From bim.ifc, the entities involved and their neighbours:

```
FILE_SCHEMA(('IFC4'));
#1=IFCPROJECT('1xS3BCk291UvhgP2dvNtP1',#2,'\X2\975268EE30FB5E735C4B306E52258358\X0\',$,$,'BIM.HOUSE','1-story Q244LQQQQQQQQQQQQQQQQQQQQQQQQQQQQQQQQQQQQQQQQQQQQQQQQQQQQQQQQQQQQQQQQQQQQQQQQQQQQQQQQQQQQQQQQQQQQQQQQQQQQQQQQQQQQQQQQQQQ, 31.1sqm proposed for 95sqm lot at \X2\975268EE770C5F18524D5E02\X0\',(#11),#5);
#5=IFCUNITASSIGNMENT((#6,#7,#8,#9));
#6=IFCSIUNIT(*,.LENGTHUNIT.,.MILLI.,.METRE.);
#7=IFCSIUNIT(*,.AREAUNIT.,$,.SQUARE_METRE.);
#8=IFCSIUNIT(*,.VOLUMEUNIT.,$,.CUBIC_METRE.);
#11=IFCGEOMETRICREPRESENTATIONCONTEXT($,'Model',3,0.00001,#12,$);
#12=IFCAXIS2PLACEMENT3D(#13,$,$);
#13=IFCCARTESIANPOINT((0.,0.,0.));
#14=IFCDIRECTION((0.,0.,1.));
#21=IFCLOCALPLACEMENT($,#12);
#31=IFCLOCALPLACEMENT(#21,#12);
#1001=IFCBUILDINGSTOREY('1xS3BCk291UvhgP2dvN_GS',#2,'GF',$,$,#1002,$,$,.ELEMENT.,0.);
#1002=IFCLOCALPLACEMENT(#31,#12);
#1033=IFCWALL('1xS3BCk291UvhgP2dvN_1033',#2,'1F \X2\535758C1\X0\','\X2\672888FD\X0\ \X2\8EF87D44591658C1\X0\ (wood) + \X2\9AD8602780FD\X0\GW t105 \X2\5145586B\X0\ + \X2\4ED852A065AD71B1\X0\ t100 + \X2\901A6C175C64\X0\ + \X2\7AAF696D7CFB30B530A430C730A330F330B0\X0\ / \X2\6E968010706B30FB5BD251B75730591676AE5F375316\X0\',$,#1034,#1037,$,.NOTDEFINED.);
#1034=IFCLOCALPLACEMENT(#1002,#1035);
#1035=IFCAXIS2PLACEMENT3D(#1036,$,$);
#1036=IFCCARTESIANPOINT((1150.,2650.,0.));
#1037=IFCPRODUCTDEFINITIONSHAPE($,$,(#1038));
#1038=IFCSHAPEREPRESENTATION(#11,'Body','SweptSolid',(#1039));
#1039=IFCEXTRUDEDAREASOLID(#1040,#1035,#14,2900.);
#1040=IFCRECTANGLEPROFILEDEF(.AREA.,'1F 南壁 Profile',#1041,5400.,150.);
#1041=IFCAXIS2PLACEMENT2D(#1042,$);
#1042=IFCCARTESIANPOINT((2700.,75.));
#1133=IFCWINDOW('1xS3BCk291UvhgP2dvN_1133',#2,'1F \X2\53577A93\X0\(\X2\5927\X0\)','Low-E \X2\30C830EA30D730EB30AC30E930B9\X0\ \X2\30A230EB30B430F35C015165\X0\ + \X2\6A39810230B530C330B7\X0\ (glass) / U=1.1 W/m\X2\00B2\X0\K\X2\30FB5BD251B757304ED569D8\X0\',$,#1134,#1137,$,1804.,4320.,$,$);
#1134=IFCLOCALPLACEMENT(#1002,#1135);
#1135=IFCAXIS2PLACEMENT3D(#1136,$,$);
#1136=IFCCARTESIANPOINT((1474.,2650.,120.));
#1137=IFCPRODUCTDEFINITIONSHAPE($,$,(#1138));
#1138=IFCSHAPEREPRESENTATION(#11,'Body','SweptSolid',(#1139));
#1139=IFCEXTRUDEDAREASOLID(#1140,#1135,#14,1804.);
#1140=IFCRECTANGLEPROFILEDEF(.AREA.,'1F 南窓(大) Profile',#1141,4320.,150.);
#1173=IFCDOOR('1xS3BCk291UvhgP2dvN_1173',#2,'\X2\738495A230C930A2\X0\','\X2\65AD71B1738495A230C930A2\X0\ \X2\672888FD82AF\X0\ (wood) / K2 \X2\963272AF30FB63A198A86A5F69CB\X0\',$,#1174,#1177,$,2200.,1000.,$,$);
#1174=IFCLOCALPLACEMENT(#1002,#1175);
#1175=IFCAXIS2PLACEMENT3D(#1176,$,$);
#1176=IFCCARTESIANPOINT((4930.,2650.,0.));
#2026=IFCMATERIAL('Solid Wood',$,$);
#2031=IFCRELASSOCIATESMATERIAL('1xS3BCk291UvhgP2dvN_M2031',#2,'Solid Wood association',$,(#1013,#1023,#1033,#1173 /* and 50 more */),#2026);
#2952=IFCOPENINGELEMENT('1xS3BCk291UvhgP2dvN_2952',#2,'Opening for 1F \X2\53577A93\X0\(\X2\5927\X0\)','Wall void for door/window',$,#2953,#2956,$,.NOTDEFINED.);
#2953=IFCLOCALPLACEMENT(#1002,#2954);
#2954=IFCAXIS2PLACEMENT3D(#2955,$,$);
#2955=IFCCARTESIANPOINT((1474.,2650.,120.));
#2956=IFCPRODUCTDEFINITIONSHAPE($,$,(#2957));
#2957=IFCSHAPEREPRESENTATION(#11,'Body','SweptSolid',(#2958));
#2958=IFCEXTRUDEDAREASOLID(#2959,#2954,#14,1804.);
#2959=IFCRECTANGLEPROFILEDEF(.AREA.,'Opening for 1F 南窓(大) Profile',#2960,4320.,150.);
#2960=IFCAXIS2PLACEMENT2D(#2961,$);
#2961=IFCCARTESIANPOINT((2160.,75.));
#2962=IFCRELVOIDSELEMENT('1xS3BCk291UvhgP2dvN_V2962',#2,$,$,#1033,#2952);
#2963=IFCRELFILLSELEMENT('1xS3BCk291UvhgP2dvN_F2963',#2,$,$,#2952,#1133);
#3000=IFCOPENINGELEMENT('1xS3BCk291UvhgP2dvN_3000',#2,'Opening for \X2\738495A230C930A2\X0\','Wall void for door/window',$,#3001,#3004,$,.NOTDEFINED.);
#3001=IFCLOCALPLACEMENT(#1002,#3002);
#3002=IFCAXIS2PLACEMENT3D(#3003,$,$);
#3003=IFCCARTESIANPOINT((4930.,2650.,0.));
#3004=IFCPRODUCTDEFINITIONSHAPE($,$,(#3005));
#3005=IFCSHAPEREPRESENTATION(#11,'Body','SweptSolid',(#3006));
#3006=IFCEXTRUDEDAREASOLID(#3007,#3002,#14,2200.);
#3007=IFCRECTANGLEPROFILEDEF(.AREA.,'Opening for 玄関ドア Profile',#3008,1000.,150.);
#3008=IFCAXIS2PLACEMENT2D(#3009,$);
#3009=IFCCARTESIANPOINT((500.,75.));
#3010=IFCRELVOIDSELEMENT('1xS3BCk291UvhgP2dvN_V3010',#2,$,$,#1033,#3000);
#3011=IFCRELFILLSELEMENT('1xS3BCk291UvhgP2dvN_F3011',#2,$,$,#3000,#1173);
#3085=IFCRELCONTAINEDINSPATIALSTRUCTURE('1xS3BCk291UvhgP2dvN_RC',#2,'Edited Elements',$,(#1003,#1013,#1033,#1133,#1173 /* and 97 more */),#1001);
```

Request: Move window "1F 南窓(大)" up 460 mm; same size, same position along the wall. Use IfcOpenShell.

```python
import numpy as np
import ifcopenshell
import ifcopenshell.api.geometry
import ifcopenshell.util.placement
import ifcopenshell.util.unit

model = ifcopenshell.open("bim.ifc")
unit_scale = ifcopenshell.util.unit.calculate_unit_scale(model)

window = model.by_guid("1xS3BCk291UvhgP2dvN_1133")
opening = window.FillsVoids[0].RelatingOpeningElement
dz = 0.46 / unit_scale

shift = np.array([0.0, 0.0, dz])
# The window is not placed relative to its opening, so move both.
for product in (opening, window):
    matrix = ifcopenshell.util.placement.get_local_placement(product.ObjectPlacement)
    matrix[:3, 3] += shift
    ifcopenshell.api.geometry.edit_object_placement(model, product=product, matrix=matrix, is_si=False)

print(f"moved by {dz * unit_scale:+.3f} m")

model.write("bim-out.ifc")
```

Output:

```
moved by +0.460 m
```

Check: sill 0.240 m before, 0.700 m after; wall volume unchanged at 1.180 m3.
